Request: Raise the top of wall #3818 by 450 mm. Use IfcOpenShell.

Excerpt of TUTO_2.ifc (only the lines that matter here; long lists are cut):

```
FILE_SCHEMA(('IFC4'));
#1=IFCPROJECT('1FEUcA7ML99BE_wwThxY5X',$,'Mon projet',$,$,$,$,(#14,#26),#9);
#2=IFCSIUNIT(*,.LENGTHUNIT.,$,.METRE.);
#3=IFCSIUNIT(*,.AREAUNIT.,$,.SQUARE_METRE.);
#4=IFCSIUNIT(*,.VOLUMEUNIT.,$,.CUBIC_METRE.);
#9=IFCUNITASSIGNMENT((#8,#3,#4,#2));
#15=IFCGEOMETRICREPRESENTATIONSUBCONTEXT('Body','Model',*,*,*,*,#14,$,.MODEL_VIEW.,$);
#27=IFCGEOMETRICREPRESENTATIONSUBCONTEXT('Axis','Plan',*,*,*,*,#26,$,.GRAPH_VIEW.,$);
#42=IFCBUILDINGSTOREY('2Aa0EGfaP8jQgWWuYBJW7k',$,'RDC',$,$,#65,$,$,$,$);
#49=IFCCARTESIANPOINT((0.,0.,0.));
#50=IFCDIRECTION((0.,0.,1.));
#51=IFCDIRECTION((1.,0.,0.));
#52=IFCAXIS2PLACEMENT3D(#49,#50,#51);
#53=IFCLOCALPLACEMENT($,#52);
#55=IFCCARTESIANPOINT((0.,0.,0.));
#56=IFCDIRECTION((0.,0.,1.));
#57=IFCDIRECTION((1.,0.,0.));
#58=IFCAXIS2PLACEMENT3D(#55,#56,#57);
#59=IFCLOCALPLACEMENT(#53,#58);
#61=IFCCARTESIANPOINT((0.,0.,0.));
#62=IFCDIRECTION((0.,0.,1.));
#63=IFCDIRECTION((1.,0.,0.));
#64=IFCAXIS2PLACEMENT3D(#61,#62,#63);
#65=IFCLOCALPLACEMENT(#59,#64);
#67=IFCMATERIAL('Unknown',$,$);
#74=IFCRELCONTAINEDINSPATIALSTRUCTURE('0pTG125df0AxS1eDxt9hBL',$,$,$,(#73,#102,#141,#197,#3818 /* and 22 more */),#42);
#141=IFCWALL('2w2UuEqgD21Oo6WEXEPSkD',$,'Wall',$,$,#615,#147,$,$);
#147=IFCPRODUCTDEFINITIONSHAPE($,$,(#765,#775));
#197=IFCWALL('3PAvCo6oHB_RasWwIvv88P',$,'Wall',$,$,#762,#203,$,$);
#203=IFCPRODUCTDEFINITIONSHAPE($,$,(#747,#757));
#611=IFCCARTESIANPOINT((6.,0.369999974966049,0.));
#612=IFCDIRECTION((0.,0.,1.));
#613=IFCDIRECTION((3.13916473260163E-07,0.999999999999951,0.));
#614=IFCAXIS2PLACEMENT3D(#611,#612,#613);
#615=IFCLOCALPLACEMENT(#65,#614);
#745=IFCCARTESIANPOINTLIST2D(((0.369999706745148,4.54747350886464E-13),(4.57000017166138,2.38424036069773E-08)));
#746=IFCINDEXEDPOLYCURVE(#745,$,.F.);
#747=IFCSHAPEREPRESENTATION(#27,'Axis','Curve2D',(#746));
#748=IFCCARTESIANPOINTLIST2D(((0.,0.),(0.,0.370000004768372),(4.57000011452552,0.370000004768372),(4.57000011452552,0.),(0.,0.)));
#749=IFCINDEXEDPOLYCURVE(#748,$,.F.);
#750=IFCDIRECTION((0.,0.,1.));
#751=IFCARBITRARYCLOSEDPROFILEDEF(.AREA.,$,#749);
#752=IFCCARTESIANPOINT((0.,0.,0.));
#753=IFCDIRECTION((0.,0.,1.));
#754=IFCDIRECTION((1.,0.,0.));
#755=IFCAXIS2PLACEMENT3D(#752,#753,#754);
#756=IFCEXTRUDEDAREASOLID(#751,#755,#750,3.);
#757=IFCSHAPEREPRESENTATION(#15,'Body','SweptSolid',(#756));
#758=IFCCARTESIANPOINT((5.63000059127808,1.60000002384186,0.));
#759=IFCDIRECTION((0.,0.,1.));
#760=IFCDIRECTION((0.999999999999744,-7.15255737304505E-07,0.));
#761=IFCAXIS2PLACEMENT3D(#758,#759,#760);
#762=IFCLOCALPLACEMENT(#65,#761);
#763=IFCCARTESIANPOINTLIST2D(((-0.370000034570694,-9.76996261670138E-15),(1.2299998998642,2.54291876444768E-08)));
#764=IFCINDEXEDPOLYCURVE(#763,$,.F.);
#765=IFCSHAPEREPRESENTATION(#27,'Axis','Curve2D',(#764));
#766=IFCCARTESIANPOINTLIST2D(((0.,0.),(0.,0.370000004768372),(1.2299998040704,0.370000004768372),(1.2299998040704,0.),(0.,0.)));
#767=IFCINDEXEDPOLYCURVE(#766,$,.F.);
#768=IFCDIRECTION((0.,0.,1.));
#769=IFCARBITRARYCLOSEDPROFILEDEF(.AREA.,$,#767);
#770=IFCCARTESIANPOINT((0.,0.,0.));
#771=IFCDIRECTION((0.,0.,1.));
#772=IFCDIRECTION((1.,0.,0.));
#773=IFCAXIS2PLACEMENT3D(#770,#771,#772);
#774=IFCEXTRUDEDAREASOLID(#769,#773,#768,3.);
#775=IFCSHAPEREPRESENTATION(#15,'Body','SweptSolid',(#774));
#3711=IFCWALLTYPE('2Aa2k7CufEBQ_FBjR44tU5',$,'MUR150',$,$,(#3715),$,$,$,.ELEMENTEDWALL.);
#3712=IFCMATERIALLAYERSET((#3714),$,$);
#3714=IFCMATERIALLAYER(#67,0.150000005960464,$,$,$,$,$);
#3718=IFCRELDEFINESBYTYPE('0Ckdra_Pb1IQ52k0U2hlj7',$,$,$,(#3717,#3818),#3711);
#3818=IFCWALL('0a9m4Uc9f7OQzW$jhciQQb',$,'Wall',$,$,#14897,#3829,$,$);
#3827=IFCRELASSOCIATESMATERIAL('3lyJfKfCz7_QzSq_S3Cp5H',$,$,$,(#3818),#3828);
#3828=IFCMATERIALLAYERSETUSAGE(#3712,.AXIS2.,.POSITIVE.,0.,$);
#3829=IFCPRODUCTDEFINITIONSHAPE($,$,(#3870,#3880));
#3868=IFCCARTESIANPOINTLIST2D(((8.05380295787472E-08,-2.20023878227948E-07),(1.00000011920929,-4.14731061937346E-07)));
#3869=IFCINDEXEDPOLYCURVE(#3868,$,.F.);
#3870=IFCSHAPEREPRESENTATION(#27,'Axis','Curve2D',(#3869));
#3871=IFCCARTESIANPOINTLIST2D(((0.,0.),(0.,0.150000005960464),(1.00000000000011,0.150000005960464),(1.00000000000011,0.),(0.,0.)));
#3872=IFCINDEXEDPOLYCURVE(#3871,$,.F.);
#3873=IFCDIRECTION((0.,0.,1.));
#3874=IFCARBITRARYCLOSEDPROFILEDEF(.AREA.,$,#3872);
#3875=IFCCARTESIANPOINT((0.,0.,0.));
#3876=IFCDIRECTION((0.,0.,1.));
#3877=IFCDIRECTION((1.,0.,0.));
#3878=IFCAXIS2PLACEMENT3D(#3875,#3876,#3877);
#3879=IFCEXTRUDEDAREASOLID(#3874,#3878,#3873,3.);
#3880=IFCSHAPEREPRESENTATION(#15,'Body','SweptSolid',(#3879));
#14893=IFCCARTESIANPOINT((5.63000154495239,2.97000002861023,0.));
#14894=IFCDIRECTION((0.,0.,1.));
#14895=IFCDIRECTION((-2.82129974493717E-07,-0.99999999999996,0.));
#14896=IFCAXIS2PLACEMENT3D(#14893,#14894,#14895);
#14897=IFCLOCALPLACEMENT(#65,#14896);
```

```python
import ifcopenshell
import ifcopenshell.geom
import ifcopenshell.util.representation
import ifcopenshell.util.shape

model = ifcopenshell.open("TUTO_2.ifc")
settings = ifcopenshell.geom.settings()


def volume(element):
    """Net volume in cubic metres, openings subtracted."""
    shape = ifcopenshell.geom.create_shape(settings, element)
    return ifcopenshell.util.shape.get_volume(shape.geometry)


wall = model.by_guid("0a9m4Uc9f7OQzW$jhciQQb")
before = volume(wall)

body = ifcopenshell.util.representation.get_representation(wall, "Model", "Body")
solid = body.Items[0]
old_height = solid.Depth
solid.Depth += 0.45
after = volume(wall)

print(f"height {old_height:g} -> {solid.Depth:g}, volume {before:.3f} -> {after:.3f} m3")

model.write("TUTO_2_edited.ifc")
```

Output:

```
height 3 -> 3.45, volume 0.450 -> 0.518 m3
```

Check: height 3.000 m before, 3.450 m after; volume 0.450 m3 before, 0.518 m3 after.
